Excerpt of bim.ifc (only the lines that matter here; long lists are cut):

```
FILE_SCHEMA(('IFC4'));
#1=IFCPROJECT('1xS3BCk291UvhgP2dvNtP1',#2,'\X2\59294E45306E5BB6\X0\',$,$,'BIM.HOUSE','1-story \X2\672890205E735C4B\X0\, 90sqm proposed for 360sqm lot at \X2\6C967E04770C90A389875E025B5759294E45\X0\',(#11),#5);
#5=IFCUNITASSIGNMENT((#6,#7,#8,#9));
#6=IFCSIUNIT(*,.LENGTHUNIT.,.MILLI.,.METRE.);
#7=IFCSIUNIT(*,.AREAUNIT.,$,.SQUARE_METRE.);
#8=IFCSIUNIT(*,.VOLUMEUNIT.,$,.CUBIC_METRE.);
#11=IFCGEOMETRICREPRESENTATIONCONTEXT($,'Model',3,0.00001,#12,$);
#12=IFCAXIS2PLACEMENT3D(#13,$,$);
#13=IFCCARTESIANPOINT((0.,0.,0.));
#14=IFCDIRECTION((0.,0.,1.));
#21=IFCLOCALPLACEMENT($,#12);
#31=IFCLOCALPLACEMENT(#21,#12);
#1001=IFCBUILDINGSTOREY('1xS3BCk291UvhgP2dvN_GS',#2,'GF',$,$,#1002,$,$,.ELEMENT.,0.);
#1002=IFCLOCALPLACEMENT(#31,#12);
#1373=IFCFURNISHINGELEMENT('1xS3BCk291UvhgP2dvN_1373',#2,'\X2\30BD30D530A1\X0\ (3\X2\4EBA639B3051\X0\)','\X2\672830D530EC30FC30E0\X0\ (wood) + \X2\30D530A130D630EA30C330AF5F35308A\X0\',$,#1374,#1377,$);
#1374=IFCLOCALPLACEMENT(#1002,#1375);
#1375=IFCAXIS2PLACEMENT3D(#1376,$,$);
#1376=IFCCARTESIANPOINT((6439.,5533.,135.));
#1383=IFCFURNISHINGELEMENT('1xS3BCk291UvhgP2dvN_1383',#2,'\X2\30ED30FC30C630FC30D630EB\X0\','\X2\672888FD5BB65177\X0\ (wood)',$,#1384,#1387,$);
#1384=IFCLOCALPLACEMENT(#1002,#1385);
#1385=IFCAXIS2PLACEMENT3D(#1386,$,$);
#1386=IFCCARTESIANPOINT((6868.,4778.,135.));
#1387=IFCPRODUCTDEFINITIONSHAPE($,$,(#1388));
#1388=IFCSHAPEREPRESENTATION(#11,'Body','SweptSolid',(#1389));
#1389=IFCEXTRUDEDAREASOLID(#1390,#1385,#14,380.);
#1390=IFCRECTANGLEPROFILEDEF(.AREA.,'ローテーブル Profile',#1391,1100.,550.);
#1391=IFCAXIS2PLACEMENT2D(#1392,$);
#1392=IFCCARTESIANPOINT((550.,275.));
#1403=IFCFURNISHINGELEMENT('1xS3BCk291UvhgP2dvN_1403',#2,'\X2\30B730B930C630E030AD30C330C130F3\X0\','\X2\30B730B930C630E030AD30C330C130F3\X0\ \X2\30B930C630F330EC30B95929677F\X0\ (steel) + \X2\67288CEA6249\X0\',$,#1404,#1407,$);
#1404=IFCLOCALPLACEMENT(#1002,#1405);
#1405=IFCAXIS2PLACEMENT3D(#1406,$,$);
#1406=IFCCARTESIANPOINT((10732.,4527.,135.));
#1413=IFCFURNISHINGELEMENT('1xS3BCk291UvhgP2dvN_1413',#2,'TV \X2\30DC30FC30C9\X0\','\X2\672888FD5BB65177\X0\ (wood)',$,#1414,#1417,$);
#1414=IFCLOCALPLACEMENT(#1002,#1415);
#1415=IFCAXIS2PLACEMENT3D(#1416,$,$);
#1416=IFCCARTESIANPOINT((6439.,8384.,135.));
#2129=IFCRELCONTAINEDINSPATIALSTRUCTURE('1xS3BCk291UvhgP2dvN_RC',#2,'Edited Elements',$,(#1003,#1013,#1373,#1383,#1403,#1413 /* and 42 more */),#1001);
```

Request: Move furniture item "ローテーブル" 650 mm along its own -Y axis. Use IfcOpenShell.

```python
import ifcopenshell
import ifcopenshell.api.geometry
import ifcopenshell.util.placement
import ifcopenshell.util.unit

model = ifcopenshell.open("bim.ifc")
unit_scale = ifcopenshell.util.unit.calculate_unit_scale(model)

item = model.by_guid("1xS3BCk291UvhgP2dvN_1383")
matrix = ifcopenshell.util.placement.get_local_placement(item.ObjectPlacement)
matrix[:3, 3] -= matrix[:3, 1] * 0.65 / unit_scale
ifcopenshell.api.geometry.edit_object_placement(model, product=item, matrix=matrix, is_si=False)

print(ifcopenshell.util.placement.get_local_placement(item.ObjectPlacement).round(3) + 0.0)

model.write("bim_v2.ifc")
```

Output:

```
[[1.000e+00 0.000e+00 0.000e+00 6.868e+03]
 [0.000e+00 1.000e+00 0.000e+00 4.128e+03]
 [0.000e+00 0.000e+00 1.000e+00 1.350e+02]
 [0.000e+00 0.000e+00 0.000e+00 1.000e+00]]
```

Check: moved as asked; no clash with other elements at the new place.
